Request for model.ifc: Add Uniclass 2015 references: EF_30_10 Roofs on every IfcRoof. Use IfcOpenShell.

First a look at what the model holds.

```python
import ifcopenshell

model = ifcopenshell.open("model.ifc")
print(model.schema)
print("classifications:", [c.Name for c in model.by_type("IfcClassification")])
for ifc_class in ("IfcDoor", "IfcRoof", "IfcStair", "IfcWall", "IfcWindow"):
    print(ifc_class, len(model.by_type(ifc_class)))
```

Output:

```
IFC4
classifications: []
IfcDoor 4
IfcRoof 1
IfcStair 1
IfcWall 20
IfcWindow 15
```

```python
import ifcopenshell
import ifcopenshell.api.classification

model = ifcopenshell.open("model.ifc")

system = ifcopenshell.api.classification.add_classification(model, classification="Uniclass 2015")

codes = {
    "IfcRoof": ("EF_30_10", "Roofs"),
}
for ifc_class, (code, name) in codes.items():
    products = model.by_type(ifc_class)
    ifcopenshell.api.classification.add_reference(
        model, products=products, classification=system, identification=code, name=name
    )
    print(code, len(products))

model.write("model_updated.ifc")
```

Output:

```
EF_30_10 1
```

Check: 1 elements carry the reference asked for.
